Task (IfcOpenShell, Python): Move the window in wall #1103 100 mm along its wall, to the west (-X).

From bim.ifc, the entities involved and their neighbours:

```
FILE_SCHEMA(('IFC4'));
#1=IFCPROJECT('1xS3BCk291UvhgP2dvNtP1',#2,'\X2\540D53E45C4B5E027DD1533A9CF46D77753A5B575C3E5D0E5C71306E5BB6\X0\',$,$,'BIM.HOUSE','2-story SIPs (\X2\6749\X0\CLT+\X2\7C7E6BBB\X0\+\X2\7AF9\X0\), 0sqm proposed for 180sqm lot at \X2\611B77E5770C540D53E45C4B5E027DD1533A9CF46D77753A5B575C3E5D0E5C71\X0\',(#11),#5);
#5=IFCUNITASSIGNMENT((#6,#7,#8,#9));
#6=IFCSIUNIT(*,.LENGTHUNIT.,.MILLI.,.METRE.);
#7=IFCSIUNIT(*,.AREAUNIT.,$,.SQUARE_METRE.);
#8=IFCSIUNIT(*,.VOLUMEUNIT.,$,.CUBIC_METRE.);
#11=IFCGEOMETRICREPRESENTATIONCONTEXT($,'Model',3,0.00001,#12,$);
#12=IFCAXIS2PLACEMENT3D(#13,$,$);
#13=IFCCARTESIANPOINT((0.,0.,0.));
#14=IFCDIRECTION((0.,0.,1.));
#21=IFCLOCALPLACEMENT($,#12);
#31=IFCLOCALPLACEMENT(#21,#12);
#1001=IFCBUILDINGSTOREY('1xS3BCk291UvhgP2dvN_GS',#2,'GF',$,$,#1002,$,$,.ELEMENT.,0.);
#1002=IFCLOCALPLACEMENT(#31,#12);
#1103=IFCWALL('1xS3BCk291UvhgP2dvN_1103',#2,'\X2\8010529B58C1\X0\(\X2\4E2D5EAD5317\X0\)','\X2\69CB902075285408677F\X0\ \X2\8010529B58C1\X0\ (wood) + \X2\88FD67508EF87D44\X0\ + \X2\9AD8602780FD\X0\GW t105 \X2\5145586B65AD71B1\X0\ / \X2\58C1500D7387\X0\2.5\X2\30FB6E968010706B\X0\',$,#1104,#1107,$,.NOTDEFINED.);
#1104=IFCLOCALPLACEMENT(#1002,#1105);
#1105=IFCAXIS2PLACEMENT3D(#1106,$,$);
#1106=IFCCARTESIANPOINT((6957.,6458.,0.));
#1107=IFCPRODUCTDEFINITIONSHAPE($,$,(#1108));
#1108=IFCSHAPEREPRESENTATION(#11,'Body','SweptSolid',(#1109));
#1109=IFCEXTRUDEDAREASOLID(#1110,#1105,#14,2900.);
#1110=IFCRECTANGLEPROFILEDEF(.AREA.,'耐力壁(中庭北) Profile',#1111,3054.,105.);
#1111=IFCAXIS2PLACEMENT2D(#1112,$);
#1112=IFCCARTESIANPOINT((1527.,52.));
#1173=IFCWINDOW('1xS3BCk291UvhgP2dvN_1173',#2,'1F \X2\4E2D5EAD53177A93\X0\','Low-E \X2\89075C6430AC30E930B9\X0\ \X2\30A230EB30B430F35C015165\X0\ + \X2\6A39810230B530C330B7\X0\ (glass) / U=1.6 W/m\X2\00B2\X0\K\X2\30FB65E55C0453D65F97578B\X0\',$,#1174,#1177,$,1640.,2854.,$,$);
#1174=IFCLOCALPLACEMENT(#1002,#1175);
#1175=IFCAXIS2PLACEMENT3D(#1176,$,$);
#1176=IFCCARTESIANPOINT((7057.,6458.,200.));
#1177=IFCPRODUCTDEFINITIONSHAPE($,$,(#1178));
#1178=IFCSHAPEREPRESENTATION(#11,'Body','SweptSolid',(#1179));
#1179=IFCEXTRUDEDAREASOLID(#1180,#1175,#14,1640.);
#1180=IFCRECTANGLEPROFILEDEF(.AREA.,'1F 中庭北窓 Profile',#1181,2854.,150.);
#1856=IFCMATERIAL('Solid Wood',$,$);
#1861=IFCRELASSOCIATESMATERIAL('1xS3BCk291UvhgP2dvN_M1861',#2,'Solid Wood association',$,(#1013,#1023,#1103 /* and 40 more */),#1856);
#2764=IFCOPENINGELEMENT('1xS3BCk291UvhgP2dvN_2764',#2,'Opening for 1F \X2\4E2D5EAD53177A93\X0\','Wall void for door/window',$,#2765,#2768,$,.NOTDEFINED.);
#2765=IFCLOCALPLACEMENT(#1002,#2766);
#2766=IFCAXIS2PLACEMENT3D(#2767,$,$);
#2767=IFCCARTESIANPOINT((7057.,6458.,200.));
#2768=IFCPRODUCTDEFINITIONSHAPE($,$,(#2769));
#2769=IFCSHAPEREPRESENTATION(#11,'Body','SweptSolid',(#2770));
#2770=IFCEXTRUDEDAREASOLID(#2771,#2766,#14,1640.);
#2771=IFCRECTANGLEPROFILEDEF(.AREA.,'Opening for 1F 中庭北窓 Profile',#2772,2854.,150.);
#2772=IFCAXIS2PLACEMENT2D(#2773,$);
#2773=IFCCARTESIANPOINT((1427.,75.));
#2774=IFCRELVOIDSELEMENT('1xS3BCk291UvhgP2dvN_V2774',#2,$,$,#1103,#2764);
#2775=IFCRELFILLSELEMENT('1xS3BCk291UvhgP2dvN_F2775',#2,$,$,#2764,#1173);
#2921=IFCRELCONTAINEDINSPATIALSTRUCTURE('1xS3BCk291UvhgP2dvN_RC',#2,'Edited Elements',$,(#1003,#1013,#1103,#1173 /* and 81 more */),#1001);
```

```python
import ifcopenshell
import ifcopenshell.api.geometry
import ifcopenshell.util.placement

model = ifcopenshell.open("bim.ifc")

window = model.by_guid("1xS3BCk291UvhgP2dvN_1173")
opening = window.FillsVoids[0].RelatingOpeningElement
wall = opening.VoidsElements[0].RelatingBuildingElement

wall_matrix = ifcopenshell.util.placement.get_local_placement(wall.ObjectPlacement)
shift = wall_matrix[:3, 0] * -100.0
before = ifcopenshell.util.placement.get_local_placement(window.ObjectPlacement)[:3, 3].copy()

# The window is not placed relative to its opening, so move both.
for product in (opening, window):
    matrix = ifcopenshell.util.placement.get_local_placement(product.ObjectPlacement)
    matrix[:3, 3] += shift
    ifcopenshell.api.geometry.edit_object_placement(model, product=product, matrix=matrix, is_si=False)

after = ifcopenshell.util.placement.get_local_placement(window.ObjectPlacement)[:3, 3]
print("window moved by", (after - before).round(3) + 0.0)

model.write("bim_v2.ifc")
```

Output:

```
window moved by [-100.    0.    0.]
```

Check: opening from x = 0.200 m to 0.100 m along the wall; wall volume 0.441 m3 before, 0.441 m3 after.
